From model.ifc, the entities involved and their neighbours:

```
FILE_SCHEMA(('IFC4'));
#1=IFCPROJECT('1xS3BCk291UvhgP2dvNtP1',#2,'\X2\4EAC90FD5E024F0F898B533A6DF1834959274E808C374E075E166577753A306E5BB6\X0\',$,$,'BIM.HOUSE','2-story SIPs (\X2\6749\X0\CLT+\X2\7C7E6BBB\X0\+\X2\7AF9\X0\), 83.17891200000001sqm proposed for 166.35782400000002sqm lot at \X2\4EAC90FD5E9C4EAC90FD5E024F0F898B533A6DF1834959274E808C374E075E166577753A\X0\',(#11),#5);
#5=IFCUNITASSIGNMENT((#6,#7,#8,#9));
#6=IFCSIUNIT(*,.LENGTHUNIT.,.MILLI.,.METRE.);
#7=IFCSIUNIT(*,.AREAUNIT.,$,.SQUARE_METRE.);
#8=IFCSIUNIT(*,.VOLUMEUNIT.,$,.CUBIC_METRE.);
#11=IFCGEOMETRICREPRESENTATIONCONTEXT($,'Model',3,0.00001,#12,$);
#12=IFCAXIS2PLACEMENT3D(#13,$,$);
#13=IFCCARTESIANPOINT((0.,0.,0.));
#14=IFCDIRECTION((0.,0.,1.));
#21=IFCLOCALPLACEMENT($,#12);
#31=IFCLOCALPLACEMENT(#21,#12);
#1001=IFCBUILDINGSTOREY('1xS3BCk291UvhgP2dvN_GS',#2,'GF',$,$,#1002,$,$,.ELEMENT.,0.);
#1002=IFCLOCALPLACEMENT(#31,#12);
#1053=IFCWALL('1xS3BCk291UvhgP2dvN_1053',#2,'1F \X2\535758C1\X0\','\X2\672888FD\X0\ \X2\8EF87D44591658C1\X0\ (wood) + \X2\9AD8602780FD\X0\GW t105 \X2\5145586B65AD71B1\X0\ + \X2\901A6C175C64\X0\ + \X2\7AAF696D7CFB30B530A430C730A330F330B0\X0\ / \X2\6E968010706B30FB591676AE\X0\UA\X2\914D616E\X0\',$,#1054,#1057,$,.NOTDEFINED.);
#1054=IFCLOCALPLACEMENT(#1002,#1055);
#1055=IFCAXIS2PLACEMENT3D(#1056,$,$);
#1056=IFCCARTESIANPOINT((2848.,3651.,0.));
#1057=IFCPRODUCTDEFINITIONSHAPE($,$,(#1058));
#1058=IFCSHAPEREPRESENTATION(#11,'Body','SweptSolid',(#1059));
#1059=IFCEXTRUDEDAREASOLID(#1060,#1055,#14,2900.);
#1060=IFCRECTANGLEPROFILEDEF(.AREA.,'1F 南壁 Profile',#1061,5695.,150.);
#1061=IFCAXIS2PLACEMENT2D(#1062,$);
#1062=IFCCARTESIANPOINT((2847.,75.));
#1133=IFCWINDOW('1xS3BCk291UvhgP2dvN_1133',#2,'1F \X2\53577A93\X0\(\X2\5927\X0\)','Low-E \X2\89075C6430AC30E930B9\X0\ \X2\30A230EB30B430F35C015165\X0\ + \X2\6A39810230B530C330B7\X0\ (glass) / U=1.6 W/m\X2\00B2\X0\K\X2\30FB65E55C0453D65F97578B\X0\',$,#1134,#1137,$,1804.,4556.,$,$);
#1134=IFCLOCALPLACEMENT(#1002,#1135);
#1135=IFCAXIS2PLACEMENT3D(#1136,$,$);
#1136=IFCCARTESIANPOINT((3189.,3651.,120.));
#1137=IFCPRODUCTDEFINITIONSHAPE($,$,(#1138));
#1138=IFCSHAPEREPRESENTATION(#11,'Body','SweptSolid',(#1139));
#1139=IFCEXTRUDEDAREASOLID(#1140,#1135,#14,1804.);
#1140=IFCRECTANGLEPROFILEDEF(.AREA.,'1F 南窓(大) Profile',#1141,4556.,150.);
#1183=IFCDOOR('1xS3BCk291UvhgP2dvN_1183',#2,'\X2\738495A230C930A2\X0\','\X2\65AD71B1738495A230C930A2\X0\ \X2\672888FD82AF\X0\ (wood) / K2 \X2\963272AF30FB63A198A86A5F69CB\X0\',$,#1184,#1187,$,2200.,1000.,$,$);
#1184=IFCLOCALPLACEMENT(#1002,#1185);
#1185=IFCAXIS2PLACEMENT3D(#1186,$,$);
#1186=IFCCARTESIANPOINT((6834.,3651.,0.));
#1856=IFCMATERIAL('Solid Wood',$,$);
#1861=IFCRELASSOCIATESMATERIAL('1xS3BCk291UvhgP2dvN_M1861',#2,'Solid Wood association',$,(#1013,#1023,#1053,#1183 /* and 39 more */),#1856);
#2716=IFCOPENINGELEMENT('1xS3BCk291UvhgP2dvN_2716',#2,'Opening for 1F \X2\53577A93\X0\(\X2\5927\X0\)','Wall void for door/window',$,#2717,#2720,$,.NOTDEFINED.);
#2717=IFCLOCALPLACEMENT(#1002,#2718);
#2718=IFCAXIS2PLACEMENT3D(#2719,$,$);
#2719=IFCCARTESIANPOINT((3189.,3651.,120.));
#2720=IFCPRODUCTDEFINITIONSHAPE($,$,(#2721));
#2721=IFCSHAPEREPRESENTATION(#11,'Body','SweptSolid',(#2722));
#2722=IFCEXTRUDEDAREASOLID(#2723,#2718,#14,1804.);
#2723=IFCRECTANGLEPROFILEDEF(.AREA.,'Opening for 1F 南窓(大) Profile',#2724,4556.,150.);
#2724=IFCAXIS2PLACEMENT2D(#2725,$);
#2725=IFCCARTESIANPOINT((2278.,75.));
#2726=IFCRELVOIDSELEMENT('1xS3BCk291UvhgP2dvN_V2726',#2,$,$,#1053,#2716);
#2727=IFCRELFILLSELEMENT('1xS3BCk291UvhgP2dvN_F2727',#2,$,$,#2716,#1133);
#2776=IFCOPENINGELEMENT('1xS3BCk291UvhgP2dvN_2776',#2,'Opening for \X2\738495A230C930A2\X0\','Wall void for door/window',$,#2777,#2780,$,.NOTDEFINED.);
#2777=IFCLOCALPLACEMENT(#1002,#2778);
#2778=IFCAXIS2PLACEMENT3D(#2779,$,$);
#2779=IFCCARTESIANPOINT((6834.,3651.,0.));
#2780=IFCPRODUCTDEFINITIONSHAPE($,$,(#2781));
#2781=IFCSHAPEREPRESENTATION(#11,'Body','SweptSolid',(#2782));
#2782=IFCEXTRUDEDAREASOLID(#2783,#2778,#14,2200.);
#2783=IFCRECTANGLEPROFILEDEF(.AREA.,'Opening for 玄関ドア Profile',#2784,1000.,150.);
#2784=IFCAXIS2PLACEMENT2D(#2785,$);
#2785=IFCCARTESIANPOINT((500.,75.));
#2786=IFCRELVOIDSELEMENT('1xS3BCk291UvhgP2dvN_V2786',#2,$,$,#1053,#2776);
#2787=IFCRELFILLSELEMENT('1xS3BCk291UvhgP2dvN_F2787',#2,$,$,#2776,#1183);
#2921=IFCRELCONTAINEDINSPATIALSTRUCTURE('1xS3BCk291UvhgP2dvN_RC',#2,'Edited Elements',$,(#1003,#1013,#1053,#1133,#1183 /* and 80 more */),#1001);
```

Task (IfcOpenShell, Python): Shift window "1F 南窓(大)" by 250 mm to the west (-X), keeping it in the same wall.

```python
import ifcopenshell
import ifcopenshell.api.geometry
import ifcopenshell.util.placement
import ifcopenshell.util.unit

model = ifcopenshell.open("model.ifc")
unit_scale = ifcopenshell.util.unit.calculate_unit_scale(model)

window = model.by_guid("1xS3BCk291UvhgP2dvN_1133")
opening = window.FillsVoids[0].RelatingOpeningElement
wall = opening.VoidsElements[0].RelatingBuildingElement

wall_matrix = ifcopenshell.util.placement.get_local_placement(wall.ObjectPlacement)
shift = wall_matrix[:3, 0] * -0.25 / unit_scale
before = ifcopenshell.util.placement.get_local_placement(window.ObjectPlacement)[:3, 3].copy()

# The window is not placed relative to its opening, so move both.
for product in (opening, window):
    matrix = ifcopenshell.util.placement.get_local_placement(product.ObjectPlacement)
    matrix[:3, 3] += shift
    ifcopenshell.api.geometry.edit_object_placement(model, product=product, matrix=matrix, is_si=False)

after = ifcopenshell.util.placement.get_local_placement(window.ObjectPlacement)[:3, 3]
print("window moved by", (after - before).round(3) + 0.0)

model.write("model_updated.ifc")
```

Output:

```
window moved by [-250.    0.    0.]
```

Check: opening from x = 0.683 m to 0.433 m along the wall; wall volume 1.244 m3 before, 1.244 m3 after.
